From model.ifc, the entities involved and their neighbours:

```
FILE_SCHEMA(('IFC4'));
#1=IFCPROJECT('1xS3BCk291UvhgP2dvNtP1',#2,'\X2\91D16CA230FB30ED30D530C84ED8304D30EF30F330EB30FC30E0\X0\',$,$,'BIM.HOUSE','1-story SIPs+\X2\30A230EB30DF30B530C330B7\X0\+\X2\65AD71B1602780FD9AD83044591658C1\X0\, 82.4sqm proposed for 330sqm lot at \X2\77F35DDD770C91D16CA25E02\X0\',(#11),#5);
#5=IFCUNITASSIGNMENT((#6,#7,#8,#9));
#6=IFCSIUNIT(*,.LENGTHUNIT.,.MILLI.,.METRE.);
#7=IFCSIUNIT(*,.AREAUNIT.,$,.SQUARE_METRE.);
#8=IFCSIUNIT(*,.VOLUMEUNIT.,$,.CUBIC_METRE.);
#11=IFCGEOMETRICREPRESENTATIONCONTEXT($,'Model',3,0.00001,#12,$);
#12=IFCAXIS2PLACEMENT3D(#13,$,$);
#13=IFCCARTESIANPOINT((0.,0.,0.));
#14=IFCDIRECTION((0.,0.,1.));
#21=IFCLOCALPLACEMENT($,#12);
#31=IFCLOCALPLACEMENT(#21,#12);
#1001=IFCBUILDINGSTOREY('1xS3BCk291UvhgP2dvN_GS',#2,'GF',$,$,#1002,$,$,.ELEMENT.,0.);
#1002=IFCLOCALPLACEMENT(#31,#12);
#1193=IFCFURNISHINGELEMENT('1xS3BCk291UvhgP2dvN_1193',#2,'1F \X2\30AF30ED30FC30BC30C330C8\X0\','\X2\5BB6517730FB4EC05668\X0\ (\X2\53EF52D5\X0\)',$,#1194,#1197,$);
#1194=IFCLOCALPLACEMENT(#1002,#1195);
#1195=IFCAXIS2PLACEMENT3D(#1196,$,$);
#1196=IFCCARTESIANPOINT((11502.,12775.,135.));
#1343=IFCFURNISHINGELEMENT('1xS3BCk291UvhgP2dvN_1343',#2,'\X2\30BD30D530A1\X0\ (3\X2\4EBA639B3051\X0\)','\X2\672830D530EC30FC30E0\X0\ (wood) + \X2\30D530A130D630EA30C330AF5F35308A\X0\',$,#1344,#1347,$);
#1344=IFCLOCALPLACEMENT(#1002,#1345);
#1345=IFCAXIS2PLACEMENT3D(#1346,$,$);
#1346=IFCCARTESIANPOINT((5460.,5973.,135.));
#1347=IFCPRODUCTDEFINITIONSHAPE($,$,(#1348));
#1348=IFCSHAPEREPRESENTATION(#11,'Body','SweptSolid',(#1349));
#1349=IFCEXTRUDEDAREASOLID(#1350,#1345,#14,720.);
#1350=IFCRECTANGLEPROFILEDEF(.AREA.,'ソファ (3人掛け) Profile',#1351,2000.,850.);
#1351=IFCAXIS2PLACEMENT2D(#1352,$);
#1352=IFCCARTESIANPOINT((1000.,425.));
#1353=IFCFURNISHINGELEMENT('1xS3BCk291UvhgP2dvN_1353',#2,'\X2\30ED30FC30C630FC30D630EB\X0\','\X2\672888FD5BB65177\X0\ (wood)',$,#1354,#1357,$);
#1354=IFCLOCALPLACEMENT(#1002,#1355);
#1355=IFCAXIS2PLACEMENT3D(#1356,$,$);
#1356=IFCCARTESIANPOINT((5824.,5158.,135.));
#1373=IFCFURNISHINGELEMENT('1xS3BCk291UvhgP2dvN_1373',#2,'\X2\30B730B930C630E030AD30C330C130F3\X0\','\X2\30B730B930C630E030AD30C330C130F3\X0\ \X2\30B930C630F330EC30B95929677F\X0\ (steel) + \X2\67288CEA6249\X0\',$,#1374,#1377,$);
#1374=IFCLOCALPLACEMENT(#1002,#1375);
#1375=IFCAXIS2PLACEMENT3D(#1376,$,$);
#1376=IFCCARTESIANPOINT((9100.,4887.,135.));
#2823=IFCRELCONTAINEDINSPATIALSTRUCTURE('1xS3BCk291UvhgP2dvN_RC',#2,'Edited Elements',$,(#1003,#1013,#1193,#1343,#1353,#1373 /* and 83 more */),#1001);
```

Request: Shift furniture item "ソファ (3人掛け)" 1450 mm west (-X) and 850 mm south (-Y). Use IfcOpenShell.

```python
import ifcopenshell
import ifcopenshell.api.geometry
import ifcopenshell.util.placement
import ifcopenshell.util.unit

model = ifcopenshell.open("model.ifc")
unit_scale = ifcopenshell.util.unit.calculate_unit_scale(model)

item = model.by_guid("1xS3BCk291UvhgP2dvN_1343")
matrix = ifcopenshell.util.placement.get_local_placement(item.ObjectPlacement)
matrix[0, 3] -= 1.45 / unit_scale
matrix[1, 3] -= 0.85 / unit_scale
ifcopenshell.api.geometry.edit_object_placement(model, product=item, matrix=matrix, is_si=False)

print(ifcopenshell.util.placement.get_local_placement(item.ObjectPlacement).round(3) + 0.0)

model.write("model_rev.ifc")
```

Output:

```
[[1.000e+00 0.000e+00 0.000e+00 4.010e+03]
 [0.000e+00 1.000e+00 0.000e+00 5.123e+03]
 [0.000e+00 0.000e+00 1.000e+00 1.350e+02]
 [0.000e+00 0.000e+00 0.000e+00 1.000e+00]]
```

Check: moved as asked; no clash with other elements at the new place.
